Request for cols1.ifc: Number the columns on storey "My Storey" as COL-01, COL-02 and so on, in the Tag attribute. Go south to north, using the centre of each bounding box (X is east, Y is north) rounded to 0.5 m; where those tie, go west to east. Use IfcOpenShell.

First a look at what the model holds.

```python
import ifcopenshell
import ifcopenshell.util.element
import ifcopenshell.util.placement

model = ifcopenshell.open("cols1.ifc")
print(model.schema)
storey = next(s for s in model.by_type("IfcBuildingStorey") if s.Name == "My Storey")
columns = [e for e in ifcopenshell.util.element.get_decomposition(storey) if e.is_a("IfcColumn")]
for e in sorted(columns, key=lambda e: e.id()):
    origin = ifcopenshell.util.placement.get_local_placement(e.ObjectPlacement)[:3, 3]
    print(e.id(), e.Tag, e.Name, origin.round(2) + 0.0, sep=" | ")
```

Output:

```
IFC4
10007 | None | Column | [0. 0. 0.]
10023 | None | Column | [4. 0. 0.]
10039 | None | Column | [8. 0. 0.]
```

```python
import ifcopenshell
import ifcopenshell.geom
import ifcopenshell.util.element
import ifcopenshell.util.shape

model = ifcopenshell.open("cols1.ifc")
settings = ifcopenshell.geom.settings()
settings.set("use-world-coords", True)


def centre(element):
    shape = ifcopenshell.geom.create_shape(settings, element)
    return ifcopenshell.util.shape.get_bbox_centroid(shape.geometry)


storey = next(s for s in model.by_type("IfcBuildingStorey") if s.Name == "My Storey")
columns = [e for e in ifcopenshell.util.element.get_decomposition(storey) if e.is_a("IfcColumn")]

# Insertion points can sit at a corner or the storey origin, so sort by the geometry (in metres).
centres = {e: centre(e) for e in columns}
columns.sort(key=lambda e: (round(centres[e][1] / 0.5), centres[e][0]))

for i, e in enumerate(columns, start=1):
    number = f"COL-{i:02d}"
    e.Tag = number
    print(e.id(), number)

model.write("cols1_edited.ifc")
```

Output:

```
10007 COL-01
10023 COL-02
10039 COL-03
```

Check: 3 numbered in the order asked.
